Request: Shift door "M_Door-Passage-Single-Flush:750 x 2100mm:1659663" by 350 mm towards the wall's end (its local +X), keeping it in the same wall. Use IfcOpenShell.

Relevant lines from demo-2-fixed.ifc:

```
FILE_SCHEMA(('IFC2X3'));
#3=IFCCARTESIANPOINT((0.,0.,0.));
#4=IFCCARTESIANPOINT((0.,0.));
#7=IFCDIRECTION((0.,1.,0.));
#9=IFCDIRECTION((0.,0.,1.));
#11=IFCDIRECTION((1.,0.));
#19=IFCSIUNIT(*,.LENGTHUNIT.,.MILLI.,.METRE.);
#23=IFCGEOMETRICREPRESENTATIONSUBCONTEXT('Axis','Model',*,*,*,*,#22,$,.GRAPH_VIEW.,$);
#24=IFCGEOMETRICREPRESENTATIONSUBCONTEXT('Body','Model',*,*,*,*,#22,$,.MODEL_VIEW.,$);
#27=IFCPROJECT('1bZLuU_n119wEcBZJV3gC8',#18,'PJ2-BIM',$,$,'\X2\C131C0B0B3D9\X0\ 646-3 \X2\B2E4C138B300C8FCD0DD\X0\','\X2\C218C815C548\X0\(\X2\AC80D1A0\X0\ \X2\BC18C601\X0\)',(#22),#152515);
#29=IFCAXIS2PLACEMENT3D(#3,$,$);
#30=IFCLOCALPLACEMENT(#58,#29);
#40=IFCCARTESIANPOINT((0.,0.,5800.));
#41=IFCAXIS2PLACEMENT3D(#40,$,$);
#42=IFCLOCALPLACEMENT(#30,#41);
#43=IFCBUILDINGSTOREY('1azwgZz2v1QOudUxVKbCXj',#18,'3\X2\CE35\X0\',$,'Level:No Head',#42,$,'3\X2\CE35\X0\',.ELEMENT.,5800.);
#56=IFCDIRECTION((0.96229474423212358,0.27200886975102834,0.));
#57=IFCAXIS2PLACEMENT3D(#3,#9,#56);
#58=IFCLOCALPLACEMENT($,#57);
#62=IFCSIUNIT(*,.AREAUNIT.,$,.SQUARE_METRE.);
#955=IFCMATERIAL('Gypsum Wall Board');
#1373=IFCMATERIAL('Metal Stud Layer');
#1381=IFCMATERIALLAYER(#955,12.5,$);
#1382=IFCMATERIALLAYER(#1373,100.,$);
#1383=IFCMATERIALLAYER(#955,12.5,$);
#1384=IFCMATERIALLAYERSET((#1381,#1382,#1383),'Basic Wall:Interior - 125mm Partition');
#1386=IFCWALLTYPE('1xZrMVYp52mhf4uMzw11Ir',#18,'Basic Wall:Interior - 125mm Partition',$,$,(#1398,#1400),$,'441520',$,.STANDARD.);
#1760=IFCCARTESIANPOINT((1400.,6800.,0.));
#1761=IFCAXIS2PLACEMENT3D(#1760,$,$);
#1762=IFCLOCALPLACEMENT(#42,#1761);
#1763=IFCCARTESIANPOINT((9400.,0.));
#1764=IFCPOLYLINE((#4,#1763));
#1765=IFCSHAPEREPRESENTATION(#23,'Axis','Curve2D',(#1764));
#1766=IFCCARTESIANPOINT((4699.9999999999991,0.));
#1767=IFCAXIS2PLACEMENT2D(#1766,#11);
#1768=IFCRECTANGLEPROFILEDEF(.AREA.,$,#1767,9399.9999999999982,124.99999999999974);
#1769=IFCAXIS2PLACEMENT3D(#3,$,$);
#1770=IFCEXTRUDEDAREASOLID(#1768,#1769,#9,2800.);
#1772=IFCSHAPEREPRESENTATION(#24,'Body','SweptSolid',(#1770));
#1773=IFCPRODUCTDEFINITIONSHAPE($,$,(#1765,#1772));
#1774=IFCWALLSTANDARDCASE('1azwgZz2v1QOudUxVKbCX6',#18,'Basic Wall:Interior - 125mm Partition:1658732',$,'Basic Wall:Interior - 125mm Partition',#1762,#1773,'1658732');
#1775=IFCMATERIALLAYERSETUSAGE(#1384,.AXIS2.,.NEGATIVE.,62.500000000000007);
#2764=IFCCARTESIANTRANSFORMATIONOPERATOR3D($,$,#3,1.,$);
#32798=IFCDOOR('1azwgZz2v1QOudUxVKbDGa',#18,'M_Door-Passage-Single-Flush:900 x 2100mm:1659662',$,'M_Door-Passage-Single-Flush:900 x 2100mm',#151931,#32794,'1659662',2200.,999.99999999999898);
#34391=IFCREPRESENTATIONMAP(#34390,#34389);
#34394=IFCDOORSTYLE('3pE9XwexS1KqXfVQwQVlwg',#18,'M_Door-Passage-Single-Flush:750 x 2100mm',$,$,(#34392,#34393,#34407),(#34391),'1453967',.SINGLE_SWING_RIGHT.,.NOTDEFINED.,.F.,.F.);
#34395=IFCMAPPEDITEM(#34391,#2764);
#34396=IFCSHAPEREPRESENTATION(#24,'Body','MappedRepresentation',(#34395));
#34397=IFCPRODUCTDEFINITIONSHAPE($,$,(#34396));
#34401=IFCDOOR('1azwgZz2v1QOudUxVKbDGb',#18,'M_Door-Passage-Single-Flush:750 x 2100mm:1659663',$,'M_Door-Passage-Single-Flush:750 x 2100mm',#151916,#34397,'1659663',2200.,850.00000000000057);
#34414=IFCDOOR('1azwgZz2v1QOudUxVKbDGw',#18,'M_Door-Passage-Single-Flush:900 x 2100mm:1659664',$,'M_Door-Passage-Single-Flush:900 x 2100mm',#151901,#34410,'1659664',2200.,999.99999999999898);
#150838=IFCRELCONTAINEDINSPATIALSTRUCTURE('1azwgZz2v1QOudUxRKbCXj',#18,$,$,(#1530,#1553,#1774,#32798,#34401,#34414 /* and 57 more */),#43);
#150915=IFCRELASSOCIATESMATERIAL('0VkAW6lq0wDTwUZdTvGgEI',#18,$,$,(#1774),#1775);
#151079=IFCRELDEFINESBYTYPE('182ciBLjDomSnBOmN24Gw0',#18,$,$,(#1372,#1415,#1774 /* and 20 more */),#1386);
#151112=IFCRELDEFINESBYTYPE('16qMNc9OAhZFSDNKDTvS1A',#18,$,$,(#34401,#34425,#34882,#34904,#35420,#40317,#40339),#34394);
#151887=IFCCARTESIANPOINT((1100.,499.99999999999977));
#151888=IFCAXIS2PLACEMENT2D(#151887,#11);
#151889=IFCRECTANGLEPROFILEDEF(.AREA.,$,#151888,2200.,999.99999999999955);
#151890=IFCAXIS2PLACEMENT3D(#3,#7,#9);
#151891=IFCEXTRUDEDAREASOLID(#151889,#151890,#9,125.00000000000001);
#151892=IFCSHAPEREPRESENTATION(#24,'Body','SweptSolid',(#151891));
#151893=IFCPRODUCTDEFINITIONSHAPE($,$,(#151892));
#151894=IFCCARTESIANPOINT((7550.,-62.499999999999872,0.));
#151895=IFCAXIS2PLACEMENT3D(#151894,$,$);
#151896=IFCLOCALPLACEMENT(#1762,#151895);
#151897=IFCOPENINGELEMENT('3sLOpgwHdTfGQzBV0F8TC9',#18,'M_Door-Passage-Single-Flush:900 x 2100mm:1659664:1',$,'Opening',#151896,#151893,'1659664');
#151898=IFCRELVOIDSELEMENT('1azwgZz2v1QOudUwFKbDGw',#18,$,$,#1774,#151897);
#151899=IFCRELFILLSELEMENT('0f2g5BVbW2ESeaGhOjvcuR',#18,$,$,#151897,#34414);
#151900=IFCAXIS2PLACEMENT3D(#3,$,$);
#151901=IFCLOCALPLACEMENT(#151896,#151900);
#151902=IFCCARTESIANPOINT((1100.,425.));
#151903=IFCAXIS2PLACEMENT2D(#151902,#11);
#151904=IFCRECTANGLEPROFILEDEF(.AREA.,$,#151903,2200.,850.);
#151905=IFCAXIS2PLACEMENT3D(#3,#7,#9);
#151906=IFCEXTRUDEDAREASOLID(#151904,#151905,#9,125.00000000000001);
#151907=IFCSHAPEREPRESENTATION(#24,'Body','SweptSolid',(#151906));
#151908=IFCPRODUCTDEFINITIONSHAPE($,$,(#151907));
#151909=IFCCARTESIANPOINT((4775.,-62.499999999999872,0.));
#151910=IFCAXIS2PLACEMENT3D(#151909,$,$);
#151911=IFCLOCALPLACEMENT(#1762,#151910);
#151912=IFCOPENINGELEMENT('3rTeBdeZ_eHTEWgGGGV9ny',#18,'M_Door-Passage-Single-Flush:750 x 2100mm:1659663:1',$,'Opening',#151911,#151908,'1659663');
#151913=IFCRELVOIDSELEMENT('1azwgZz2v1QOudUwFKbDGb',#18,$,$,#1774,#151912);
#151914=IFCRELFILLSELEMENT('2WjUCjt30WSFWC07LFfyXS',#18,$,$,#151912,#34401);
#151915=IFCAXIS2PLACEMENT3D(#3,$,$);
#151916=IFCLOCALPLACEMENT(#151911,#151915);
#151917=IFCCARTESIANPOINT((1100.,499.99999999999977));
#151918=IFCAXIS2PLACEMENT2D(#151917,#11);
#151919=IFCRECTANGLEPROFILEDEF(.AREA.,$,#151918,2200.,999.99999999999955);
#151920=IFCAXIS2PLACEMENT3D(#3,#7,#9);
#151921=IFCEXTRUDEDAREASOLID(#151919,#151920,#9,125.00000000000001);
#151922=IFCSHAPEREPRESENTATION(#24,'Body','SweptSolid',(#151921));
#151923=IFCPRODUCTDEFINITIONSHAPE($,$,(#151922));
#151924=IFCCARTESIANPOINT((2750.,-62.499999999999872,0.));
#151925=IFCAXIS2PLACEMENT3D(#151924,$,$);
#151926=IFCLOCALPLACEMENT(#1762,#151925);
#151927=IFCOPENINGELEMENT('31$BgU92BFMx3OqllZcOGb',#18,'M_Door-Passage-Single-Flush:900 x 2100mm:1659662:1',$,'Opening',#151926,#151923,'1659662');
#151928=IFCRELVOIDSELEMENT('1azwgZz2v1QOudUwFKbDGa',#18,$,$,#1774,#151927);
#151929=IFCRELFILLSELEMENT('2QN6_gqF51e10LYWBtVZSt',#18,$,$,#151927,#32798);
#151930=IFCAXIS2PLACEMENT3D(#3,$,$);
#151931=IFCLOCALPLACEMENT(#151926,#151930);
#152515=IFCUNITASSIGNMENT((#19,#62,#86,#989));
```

```python
import ifcopenshell
import ifcopenshell.api.geometry
import ifcopenshell.util.placement
import ifcopenshell.util.unit

model = ifcopenshell.open("demo-2-fixed.ifc")
unit_scale = ifcopenshell.util.unit.calculate_unit_scale(model)

door = model.by_guid("1azwgZz2v1QOudUxVKbDGb")
opening = door.FillsVoids[0].RelatingOpeningElement
wall = opening.VoidsElements[0].RelatingBuildingElement

wall_matrix = ifcopenshell.util.placement.get_local_placement(wall.ObjectPlacement)
shift = wall_matrix[:3, 0] * 0.35 / unit_scale
before = ifcopenshell.util.placement.get_local_placement(door.ObjectPlacement)[:3, 3].copy()

# The door is placed relative to its opening, so it follows when the opening moves.
matrix = ifcopenshell.util.placement.get_local_placement(opening.ObjectPlacement)
matrix[:3, 3] += shift
ifcopenshell.api.geometry.edit_object_placement(
    model, product=opening, matrix=matrix, is_si=False, should_transform_children=True
)

after = ifcopenshell.util.placement.get_local_placement(door.ObjectPlacement)[:3, 3]
print("door moved by", (after - before).round(3) + 0.0)

model.write("demo-2-fixed_rev.ifc")
```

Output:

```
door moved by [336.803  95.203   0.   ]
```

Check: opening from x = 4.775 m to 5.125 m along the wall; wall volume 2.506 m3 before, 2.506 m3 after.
